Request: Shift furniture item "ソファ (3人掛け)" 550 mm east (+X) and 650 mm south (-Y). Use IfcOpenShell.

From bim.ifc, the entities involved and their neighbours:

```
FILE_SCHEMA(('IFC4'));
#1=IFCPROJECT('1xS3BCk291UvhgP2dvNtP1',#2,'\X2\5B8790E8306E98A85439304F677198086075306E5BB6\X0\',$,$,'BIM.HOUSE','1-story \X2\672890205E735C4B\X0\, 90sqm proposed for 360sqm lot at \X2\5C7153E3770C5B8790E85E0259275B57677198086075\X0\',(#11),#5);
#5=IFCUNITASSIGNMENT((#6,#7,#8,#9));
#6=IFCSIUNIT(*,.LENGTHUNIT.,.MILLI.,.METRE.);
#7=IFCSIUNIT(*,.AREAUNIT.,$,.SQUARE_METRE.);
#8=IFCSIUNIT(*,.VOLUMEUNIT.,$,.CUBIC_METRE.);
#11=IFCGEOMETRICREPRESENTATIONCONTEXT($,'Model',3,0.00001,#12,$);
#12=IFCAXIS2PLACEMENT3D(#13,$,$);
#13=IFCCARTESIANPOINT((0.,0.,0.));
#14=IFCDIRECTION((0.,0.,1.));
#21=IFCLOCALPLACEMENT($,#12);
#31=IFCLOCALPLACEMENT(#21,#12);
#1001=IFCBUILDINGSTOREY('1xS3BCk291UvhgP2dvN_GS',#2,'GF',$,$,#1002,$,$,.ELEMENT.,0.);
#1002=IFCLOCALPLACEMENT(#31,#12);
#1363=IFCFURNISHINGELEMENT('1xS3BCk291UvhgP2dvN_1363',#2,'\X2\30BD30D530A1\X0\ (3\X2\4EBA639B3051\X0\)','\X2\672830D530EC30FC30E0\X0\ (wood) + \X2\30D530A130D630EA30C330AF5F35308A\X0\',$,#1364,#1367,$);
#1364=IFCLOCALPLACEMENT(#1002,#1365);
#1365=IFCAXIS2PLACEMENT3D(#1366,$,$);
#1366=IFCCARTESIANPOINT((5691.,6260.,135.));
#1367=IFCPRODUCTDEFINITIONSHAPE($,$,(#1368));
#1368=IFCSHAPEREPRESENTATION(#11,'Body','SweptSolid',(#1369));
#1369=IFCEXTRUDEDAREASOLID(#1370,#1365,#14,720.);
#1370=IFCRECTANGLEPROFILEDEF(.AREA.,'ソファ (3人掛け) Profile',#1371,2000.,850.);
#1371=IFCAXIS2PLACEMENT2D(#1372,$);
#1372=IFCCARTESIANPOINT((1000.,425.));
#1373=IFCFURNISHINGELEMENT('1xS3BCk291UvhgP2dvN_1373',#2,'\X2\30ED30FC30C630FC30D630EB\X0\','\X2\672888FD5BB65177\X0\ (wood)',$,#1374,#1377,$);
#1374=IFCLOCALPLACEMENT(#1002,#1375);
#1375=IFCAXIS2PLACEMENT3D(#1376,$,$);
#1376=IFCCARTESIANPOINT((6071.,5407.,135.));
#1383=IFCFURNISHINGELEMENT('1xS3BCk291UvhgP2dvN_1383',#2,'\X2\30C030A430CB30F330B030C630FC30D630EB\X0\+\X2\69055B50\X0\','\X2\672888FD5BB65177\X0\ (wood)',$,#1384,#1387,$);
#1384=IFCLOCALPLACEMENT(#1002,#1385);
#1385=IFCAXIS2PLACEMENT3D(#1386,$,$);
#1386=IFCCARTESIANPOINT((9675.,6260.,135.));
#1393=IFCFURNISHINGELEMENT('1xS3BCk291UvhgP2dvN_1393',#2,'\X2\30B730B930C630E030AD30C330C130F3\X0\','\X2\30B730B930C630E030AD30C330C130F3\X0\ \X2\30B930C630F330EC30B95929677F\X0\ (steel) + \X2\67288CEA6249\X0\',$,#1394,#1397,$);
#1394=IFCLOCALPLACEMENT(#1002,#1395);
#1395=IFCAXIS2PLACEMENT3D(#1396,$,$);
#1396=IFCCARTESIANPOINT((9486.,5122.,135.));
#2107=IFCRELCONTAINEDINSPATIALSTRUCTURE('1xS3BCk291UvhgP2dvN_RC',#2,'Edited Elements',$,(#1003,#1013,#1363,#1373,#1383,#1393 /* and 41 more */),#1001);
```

```python
import ifcopenshell
import ifcopenshell.api.geometry
import ifcopenshell.util.placement

model = ifcopenshell.open("bim.ifc")

item = model.by_guid("1xS3BCk291UvhgP2dvN_1363")
matrix = ifcopenshell.util.placement.get_local_placement(item.ObjectPlacement)
matrix[0, 3] += 550.0
matrix[1, 3] -= 650.0
ifcopenshell.api.geometry.edit_object_placement(model, product=item, matrix=matrix, is_si=False)

print(ifcopenshell.util.placement.get_local_placement(item.ObjectPlacement).round(3) + 0.0)

model.write("bim_v2.ifc")
```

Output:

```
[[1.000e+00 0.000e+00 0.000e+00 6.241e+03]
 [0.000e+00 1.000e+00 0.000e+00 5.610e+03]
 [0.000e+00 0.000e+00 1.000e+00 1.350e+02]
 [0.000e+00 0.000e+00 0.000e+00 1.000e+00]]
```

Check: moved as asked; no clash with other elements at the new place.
